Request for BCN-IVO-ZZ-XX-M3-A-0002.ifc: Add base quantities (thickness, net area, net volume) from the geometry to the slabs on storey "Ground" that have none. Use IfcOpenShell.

First a look at what the model holds.

```python
import ifcopenshell
import ifcopenshell.util.element
import ifcopenshell.util.unit

model = ifcopenshell.open("BCN-IVO-ZZ-XX-M3-A-0002.ifc")
print(model.schema)
for unit_type in ("LENGTHUNIT", "AREAUNIT", "VOLUMEUNIT"):
    print(unit_type, ifcopenshell.util.unit.calculate_unit_scale(model, unit_type))
storey = next(s for s in model.by_type("IfcBuildingStorey") if s.Name == "Ground")
slabs = [e for e in ifcopenshell.util.element.get_decomposition(storey) if e.is_a("IfcSlab")]
for e in sorted(slabs, key=lambda e: e.id()):
    print(e.id(), e.is_a(), e.Name, list(ifcopenshell.util.element.get_psets(e, qtos_only=True)), sep=" | ")
```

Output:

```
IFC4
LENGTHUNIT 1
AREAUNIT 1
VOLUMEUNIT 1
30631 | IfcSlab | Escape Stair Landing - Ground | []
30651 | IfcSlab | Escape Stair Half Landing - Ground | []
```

```python
import ifcopenshell
import ifcopenshell.api.pset
import ifcopenshell.geom
import ifcopenshell.util.element
import ifcopenshell.util.shape
import ifcopenshell.util.unit

model = ifcopenshell.open("BCN-IVO-ZZ-XX-M3-A-0002.ifc")
unit_scale = ifcopenshell.util.unit.calculate_unit_scale(model)
area_scale = ifcopenshell.util.unit.calculate_unit_scale(model, "AREAUNIT")
volume_scale = ifcopenshell.util.unit.calculate_unit_scale(model, "VOLUMEUNIT")
settings = ifcopenshell.geom.settings()

storey = next(s for s in model.by_type("IfcBuildingStorey") if s.Name == "Ground")
slabs = [e for e in ifcopenshell.util.element.get_decomposition(storey) if e.is_a("IfcSlab")]

for e in sorted(slabs, key=lambda e: e.id()):
    if ifcopenshell.util.element.get_psets(e, qtos_only=True, should_inherit=False):
        continue
    # Geometry comes back in metres, in the element's own axes.
    shape = ifcopenshell.geom.create_shape(settings, e)
    values = {
        "Width": ifcopenshell.util.shape.get_z(shape.geometry) / unit_scale,
        "NetArea": ifcopenshell.util.shape.get_footprint_area(shape.geometry) / area_scale,
        "NetVolume": ifcopenshell.util.shape.get_volume(shape.geometry) / volume_scale,
    }
    qto = ifcopenshell.api.pset.add_qto(model, product=e, name="Qto_SlabBaseQuantities")
    ifcopenshell.api.pset.edit_qto(model, qto=qto, properties=values)
    print(e.id(), {k: round(v, 3) for k, v in values.items()})

model.write("BCN-IVO-ZZ-XX-M3-A-0002_v2.ifc")
```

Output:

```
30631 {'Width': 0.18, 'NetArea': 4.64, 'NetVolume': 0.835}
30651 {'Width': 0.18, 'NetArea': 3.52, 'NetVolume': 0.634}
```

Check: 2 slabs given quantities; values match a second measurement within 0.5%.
